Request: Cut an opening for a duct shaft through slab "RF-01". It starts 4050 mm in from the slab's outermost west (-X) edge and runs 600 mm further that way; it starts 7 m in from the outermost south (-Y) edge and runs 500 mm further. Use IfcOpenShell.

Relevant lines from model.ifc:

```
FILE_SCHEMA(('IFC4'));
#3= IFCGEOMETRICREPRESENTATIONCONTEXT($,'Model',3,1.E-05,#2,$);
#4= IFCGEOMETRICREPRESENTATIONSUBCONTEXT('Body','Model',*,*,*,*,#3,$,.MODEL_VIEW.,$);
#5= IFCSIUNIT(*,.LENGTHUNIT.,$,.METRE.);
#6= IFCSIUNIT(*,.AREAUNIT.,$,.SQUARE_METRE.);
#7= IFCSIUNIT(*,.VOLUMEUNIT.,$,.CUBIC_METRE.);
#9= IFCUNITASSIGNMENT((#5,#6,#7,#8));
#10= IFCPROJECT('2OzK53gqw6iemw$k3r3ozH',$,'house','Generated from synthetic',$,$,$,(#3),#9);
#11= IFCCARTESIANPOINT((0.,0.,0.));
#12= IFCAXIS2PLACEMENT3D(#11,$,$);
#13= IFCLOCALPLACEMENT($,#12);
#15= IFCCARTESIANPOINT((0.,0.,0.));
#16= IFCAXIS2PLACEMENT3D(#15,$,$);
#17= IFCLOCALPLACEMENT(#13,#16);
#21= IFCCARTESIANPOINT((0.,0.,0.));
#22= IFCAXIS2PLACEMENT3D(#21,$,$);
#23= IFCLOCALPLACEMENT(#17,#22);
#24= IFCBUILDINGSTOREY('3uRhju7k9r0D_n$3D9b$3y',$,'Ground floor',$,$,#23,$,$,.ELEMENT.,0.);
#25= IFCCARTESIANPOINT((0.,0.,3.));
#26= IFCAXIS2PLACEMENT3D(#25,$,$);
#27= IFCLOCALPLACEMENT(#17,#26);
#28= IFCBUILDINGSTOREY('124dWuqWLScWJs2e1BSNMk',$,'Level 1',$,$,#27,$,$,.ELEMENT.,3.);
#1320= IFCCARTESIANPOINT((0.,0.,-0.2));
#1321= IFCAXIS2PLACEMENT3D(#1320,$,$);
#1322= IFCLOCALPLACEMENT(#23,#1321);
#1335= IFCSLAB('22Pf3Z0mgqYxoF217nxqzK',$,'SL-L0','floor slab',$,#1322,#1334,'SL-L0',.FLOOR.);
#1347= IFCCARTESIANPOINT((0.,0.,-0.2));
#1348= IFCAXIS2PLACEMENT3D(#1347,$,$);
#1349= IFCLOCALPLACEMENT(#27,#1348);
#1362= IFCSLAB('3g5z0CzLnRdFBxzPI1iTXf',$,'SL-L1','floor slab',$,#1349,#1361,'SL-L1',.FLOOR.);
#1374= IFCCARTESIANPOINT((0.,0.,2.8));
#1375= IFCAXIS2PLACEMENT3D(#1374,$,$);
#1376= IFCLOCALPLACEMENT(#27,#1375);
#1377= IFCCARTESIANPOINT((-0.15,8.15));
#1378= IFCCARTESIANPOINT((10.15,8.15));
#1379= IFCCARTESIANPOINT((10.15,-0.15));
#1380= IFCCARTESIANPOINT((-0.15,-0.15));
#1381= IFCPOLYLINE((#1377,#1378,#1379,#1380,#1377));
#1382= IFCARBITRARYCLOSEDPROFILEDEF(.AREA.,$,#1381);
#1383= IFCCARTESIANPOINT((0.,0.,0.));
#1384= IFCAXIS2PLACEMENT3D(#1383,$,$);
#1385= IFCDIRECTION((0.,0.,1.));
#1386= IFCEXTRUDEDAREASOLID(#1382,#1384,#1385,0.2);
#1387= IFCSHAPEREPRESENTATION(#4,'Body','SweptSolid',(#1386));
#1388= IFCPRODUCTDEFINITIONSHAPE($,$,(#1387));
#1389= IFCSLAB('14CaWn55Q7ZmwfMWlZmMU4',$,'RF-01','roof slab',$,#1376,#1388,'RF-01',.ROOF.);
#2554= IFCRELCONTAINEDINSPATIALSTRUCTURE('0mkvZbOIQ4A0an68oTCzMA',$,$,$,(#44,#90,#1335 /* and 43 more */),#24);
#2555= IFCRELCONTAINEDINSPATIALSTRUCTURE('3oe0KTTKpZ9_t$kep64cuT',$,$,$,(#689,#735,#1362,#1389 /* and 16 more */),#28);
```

```python
import numpy as np
import ifcopenshell
import ifcopenshell.api.feature
import ifcopenshell.api.geometry
import ifcopenshell.api.root
import ifcopenshell.geom
import ifcopenshell.util.placement
import ifcopenshell.util.representation
import ifcopenshell.util.shape
import ifcopenshell.util.unit

model = ifcopenshell.open("model.ifc")
unit_scale = ifcopenshell.util.unit.calculate_unit_scale(model)
settings = ifcopenshell.geom.settings()


def volume(element):
    """Net volume in cubic metres, openings subtracted."""
    shape = ifcopenshell.geom.create_shape(settings, element)
    return ifcopenshell.util.shape.get_volume(shape.geometry)


slab = model.by_guid("14CaWn55Q7ZmwfMWlZmMU4")
before = volume(slab)

# Extent in the slab's own axes, in metres. The edges named are its -X and -Y sides.
slab_shape = ifcopenshell.geom.create_shape(settings, slab)
vertices = ifcopenshell.util.shape.get_vertices(slab_shape.geometry)
x_min, y_min, bottom = vertices.min(axis=0)
top = vertices[:, 2].max()

opening = ifcopenshell.api.root.create_entity(model, ifc_class="IfcOpeningElement", name="Duct shaft opening", predefined_type="OPENING")
context = ifcopenshell.util.representation.get_context(model, "Model", "Body", "MODEL_VIEW")
width, depth = 0.6, 0.5
outline = [(0.0, 0.0), (width, 0.0), (width, depth), (0.0, depth), (0.0, 0.0)]
# Overshoot both faces by 50 mm so the cut is clean.
shape = ifcopenshell.api.geometry.add_slab_representation(
    model, context=context, depth=top - bottom + 0.1, polyline=outline
)
ifcopenshell.api.geometry.assign_representation(model, product=opening, representation=shape)

matrix = ifcopenshell.util.placement.get_local_placement(slab.ObjectPlacement)
matrix[:, 3] = matrix @ np.append(np.array([x_min + 4.05, y_min + 7, bottom - 0.05]) / unit_scale, 1.0)
ifcopenshell.api.geometry.edit_object_placement(model, product=opening, matrix=matrix, is_si=False)
ifcopenshell.api.feature.add_feature(model, feature=opening, element=slab)

after = volume(slab)

print(f"slab volume {before:.3f} -> {after:.3f} m3")

model.write("model-out.ifc")
```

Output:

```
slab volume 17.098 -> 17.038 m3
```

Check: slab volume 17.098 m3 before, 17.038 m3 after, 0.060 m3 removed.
